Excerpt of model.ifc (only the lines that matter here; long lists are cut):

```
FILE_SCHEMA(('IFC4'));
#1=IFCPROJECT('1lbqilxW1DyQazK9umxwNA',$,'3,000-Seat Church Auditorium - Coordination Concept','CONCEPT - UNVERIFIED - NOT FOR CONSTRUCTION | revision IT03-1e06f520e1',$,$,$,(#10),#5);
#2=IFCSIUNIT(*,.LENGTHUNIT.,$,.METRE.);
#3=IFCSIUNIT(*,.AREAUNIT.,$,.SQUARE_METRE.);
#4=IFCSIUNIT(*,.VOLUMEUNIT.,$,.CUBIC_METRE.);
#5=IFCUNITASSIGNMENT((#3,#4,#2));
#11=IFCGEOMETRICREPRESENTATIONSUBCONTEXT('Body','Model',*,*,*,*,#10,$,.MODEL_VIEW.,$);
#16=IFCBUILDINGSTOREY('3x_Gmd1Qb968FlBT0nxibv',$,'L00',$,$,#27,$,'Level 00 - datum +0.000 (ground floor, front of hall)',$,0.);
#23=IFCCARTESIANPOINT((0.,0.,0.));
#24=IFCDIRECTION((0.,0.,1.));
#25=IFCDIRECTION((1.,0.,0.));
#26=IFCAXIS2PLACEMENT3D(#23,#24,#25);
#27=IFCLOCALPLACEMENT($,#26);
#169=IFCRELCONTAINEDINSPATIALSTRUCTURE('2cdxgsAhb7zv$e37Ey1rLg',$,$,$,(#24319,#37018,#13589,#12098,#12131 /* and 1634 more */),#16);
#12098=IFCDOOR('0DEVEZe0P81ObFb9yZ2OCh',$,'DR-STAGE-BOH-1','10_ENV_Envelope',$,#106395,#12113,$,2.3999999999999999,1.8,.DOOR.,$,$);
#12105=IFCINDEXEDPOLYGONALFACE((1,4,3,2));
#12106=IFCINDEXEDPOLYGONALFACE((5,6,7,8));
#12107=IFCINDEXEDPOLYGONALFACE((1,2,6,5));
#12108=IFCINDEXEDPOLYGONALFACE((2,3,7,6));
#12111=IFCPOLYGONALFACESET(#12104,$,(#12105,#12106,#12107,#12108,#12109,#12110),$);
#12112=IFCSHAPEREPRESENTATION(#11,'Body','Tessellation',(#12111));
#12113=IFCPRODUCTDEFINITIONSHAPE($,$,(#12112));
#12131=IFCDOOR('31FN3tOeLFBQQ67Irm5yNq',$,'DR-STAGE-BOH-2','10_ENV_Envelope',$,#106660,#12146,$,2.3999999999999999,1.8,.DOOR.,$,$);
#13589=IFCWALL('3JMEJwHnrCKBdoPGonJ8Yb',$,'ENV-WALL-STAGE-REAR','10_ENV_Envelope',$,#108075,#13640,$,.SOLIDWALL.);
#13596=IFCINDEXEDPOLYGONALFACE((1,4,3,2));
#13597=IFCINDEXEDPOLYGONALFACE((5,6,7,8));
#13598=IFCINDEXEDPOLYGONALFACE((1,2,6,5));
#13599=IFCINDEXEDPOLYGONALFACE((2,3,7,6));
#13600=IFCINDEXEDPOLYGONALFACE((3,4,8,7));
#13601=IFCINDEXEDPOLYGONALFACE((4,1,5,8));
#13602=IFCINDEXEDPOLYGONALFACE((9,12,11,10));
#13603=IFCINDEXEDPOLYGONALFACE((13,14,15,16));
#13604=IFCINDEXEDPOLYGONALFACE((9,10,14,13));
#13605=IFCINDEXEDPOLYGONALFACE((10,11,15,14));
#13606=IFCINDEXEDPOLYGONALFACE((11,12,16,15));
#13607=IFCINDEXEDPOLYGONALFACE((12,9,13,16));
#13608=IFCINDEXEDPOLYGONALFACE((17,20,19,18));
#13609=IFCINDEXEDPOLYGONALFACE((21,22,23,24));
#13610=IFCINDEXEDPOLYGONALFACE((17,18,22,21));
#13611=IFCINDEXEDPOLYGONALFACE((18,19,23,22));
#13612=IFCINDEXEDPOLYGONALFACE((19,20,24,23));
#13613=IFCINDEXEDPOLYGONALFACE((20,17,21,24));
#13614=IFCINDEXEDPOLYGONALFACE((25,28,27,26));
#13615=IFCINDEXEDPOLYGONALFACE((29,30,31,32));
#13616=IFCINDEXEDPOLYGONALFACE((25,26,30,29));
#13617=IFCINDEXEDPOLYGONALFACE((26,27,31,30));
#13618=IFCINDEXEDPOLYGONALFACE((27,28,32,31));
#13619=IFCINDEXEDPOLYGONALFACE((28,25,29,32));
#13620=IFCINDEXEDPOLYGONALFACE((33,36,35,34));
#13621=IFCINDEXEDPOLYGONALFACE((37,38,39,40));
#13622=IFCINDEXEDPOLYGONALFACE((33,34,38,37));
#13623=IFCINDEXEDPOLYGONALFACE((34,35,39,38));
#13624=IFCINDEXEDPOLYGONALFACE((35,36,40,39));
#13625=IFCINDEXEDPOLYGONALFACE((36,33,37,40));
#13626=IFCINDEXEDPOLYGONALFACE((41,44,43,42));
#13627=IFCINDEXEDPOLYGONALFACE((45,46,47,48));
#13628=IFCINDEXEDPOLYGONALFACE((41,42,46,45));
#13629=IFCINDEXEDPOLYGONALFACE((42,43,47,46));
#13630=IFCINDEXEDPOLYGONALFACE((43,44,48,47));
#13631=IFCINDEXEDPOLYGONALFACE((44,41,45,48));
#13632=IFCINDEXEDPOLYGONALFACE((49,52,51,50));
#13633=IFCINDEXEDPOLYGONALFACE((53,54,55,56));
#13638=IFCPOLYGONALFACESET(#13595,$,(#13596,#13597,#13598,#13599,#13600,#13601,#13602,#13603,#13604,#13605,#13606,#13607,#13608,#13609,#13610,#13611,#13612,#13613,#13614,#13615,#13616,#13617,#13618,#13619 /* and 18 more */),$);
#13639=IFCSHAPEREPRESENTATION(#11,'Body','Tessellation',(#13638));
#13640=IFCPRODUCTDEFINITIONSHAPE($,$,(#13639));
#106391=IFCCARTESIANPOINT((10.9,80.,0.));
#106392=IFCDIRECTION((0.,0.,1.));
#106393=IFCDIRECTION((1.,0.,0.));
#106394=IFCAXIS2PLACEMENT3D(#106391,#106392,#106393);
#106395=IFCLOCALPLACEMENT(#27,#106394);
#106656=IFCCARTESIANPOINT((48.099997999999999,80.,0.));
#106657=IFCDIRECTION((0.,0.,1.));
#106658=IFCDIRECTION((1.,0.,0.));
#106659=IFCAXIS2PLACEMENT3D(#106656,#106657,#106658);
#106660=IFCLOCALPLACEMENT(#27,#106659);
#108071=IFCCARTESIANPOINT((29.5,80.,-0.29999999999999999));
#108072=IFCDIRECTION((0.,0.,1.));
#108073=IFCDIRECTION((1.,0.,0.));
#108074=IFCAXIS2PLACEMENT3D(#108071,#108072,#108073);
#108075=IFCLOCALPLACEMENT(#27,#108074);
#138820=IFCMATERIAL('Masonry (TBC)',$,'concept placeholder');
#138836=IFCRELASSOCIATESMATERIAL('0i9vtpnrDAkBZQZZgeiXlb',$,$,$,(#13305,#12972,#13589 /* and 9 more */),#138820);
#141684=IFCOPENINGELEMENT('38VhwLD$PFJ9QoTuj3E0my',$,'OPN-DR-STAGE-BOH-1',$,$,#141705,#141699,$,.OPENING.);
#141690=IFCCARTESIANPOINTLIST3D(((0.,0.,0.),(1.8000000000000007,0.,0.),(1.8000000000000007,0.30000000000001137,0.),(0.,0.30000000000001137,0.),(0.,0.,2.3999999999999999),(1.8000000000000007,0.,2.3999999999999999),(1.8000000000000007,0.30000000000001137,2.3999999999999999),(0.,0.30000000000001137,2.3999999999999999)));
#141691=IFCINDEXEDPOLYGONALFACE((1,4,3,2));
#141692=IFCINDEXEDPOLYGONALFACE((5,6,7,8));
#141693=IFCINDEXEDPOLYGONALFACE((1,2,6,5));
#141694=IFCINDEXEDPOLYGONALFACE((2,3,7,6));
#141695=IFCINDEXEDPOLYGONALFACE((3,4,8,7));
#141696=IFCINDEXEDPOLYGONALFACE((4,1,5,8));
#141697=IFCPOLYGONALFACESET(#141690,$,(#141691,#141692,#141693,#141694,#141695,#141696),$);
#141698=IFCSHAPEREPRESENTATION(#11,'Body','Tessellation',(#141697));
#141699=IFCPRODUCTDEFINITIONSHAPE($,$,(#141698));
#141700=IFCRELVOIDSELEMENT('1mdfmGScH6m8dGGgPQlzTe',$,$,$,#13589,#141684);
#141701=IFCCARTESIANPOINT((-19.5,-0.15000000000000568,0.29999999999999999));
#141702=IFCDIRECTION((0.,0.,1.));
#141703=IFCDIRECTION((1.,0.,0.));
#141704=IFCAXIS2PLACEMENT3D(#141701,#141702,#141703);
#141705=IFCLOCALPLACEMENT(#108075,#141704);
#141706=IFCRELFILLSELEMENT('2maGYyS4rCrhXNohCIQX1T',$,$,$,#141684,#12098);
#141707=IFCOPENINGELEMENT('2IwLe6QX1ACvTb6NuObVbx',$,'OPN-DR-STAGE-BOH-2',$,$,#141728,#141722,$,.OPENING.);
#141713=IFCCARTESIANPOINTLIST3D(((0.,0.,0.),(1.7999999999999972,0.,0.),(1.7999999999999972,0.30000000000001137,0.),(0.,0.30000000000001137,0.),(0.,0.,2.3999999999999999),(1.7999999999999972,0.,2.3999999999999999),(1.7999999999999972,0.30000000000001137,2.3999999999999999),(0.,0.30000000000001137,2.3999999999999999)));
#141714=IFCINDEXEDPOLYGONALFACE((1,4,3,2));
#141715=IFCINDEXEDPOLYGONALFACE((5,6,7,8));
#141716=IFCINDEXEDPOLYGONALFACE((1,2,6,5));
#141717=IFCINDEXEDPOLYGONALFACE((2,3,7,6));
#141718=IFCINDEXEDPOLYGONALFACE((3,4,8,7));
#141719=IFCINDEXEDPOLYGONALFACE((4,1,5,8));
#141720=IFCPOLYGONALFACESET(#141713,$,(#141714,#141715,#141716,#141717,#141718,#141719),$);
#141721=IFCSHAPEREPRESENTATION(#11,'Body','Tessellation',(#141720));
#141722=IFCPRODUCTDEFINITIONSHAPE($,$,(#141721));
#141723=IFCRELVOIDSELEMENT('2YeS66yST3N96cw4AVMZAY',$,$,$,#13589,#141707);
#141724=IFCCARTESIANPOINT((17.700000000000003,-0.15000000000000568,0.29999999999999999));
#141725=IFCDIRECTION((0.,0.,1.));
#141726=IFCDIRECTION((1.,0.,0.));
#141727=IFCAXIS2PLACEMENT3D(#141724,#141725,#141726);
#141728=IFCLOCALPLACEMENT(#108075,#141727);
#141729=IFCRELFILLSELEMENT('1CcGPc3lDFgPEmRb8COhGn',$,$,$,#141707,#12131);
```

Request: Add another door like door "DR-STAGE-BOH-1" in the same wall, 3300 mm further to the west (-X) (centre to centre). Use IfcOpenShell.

```python
import ifcopenshell
import ifcopenshell.api.feature
import ifcopenshell.api.geometry
import ifcopenshell.api.root
import ifcopenshell.geom
import ifcopenshell.util.element
import ifcopenshell.util.placement
import ifcopenshell.util.shape

model = ifcopenshell.open("model.ifc")
settings = ifcopenshell.geom.settings()


def volume(element):
    """Net volume in cubic metres, openings subtracted."""
    shape = ifcopenshell.geom.create_shape(settings, element)
    return ifcopenshell.util.shape.get_volume(shape.geometry)


door = model.by_guid("0DEVEZe0P81ObFb9yZ2OCh")
opening = door.FillsVoids[0].RelatingOpeningElement
wall = opening.VoidsElements[0].RelatingBuildingElement
before = volume(wall)
shift = ifcopenshell.util.placement.get_local_placement(wall.ObjectPlacement)[:3, 0] * -3.3

# copy_class copies the void relationship, type, container and properties, but no geometry.
new_opening = ifcopenshell.api.root.copy_class(model, product=opening)
new_opening.Representation = ifcopenshell.util.element.copy_deep(
    model, opening.Representation, exclude=["IfcGeometricRepresentationContext", "IfcRepresentationMap"]
)
new_door = ifcopenshell.api.root.copy_class(model, product=door)
new_door.Representation = ifcopenshell.util.element.copy_deep(
    model, door.Representation, exclude=["IfcGeometricRepresentationContext", "IfcRepresentationMap"]
)
ifcopenshell.api.feature.add_filling(model, opening=new_opening, element=new_door)

for old, new in ((opening, new_opening), (door, new_door)):
    matrix = ifcopenshell.util.placement.get_local_placement(old.ObjectPlacement)
    matrix[:3, 3] += shift
    ifcopenshell.api.geometry.edit_object_placement(model, product=new, matrix=matrix, is_si=False)

after = volume(wall)

print(f"wall volume {before:.3f} -> {after:.3f} m3")

model.write("model_rev.ifc")
```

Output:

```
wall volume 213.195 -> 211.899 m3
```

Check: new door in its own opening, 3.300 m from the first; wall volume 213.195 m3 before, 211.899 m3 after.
